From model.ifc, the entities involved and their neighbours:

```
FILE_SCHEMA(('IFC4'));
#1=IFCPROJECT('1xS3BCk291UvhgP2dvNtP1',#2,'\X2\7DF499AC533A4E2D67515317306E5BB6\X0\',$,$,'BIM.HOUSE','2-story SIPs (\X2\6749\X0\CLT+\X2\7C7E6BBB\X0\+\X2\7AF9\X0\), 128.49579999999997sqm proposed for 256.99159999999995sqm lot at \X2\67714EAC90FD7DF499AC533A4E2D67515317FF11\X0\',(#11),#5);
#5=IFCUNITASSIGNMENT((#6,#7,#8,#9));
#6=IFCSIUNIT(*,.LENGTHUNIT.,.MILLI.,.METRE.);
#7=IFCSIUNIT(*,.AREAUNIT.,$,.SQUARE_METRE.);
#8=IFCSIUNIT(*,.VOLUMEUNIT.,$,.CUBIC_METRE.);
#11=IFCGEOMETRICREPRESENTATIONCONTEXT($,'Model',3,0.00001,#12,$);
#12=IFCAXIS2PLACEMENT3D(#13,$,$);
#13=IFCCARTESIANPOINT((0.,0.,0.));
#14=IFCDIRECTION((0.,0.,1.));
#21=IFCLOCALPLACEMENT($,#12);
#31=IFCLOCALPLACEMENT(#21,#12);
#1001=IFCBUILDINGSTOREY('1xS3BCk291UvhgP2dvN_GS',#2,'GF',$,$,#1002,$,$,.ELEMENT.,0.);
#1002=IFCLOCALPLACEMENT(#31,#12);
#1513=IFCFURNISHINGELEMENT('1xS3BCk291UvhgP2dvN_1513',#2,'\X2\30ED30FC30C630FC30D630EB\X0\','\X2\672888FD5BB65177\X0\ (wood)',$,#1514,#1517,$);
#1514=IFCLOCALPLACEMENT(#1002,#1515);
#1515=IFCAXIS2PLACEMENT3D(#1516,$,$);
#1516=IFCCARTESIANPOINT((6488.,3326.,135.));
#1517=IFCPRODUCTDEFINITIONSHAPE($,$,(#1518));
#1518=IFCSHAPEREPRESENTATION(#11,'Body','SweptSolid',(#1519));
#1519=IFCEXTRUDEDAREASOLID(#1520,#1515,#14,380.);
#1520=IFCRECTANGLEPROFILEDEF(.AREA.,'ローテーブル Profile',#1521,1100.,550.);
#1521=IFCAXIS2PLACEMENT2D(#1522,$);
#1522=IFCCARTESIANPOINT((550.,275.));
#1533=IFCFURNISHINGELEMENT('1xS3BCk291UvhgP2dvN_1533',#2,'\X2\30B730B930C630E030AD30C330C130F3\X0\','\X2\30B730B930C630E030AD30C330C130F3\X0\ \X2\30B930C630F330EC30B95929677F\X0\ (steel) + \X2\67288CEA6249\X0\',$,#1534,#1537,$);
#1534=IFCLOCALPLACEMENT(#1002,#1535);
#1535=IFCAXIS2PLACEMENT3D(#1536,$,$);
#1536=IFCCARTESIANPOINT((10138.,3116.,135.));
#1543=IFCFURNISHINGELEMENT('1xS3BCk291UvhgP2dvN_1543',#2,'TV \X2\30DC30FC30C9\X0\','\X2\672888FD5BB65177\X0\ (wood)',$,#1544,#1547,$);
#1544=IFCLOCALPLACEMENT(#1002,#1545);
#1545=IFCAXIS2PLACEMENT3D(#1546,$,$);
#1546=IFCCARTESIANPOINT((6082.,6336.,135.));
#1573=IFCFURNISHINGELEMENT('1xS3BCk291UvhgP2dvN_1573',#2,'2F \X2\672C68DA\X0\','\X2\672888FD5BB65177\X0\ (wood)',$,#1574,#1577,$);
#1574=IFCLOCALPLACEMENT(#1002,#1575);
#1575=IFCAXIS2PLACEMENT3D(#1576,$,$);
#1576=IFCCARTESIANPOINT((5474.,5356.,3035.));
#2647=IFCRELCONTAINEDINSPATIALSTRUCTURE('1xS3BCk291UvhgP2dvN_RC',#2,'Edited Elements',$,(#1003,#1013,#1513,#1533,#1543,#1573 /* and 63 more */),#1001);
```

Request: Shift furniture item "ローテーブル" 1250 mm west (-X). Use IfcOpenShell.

```python
import ifcopenshell
import ifcopenshell.api.geometry
import ifcopenshell.util.placement
import ifcopenshell.util.unit

model = ifcopenshell.open("model.ifc")
unit_scale = ifcopenshell.util.unit.calculate_unit_scale(model)

item = model.by_guid("1xS3BCk291UvhgP2dvN_1513")
matrix = ifcopenshell.util.placement.get_local_placement(item.ObjectPlacement)
matrix[0, 3] -= 1.25 / unit_scale
ifcopenshell.api.geometry.edit_object_placement(model, product=item, matrix=matrix, is_si=False)

print(ifcopenshell.util.placement.get_local_placement(item.ObjectPlacement).round(3) + 0.0)

model.write("model-out.ifc")
```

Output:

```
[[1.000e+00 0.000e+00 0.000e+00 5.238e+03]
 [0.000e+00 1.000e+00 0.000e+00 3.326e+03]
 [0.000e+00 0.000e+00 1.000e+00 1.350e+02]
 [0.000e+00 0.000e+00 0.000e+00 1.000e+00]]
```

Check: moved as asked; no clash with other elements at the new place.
